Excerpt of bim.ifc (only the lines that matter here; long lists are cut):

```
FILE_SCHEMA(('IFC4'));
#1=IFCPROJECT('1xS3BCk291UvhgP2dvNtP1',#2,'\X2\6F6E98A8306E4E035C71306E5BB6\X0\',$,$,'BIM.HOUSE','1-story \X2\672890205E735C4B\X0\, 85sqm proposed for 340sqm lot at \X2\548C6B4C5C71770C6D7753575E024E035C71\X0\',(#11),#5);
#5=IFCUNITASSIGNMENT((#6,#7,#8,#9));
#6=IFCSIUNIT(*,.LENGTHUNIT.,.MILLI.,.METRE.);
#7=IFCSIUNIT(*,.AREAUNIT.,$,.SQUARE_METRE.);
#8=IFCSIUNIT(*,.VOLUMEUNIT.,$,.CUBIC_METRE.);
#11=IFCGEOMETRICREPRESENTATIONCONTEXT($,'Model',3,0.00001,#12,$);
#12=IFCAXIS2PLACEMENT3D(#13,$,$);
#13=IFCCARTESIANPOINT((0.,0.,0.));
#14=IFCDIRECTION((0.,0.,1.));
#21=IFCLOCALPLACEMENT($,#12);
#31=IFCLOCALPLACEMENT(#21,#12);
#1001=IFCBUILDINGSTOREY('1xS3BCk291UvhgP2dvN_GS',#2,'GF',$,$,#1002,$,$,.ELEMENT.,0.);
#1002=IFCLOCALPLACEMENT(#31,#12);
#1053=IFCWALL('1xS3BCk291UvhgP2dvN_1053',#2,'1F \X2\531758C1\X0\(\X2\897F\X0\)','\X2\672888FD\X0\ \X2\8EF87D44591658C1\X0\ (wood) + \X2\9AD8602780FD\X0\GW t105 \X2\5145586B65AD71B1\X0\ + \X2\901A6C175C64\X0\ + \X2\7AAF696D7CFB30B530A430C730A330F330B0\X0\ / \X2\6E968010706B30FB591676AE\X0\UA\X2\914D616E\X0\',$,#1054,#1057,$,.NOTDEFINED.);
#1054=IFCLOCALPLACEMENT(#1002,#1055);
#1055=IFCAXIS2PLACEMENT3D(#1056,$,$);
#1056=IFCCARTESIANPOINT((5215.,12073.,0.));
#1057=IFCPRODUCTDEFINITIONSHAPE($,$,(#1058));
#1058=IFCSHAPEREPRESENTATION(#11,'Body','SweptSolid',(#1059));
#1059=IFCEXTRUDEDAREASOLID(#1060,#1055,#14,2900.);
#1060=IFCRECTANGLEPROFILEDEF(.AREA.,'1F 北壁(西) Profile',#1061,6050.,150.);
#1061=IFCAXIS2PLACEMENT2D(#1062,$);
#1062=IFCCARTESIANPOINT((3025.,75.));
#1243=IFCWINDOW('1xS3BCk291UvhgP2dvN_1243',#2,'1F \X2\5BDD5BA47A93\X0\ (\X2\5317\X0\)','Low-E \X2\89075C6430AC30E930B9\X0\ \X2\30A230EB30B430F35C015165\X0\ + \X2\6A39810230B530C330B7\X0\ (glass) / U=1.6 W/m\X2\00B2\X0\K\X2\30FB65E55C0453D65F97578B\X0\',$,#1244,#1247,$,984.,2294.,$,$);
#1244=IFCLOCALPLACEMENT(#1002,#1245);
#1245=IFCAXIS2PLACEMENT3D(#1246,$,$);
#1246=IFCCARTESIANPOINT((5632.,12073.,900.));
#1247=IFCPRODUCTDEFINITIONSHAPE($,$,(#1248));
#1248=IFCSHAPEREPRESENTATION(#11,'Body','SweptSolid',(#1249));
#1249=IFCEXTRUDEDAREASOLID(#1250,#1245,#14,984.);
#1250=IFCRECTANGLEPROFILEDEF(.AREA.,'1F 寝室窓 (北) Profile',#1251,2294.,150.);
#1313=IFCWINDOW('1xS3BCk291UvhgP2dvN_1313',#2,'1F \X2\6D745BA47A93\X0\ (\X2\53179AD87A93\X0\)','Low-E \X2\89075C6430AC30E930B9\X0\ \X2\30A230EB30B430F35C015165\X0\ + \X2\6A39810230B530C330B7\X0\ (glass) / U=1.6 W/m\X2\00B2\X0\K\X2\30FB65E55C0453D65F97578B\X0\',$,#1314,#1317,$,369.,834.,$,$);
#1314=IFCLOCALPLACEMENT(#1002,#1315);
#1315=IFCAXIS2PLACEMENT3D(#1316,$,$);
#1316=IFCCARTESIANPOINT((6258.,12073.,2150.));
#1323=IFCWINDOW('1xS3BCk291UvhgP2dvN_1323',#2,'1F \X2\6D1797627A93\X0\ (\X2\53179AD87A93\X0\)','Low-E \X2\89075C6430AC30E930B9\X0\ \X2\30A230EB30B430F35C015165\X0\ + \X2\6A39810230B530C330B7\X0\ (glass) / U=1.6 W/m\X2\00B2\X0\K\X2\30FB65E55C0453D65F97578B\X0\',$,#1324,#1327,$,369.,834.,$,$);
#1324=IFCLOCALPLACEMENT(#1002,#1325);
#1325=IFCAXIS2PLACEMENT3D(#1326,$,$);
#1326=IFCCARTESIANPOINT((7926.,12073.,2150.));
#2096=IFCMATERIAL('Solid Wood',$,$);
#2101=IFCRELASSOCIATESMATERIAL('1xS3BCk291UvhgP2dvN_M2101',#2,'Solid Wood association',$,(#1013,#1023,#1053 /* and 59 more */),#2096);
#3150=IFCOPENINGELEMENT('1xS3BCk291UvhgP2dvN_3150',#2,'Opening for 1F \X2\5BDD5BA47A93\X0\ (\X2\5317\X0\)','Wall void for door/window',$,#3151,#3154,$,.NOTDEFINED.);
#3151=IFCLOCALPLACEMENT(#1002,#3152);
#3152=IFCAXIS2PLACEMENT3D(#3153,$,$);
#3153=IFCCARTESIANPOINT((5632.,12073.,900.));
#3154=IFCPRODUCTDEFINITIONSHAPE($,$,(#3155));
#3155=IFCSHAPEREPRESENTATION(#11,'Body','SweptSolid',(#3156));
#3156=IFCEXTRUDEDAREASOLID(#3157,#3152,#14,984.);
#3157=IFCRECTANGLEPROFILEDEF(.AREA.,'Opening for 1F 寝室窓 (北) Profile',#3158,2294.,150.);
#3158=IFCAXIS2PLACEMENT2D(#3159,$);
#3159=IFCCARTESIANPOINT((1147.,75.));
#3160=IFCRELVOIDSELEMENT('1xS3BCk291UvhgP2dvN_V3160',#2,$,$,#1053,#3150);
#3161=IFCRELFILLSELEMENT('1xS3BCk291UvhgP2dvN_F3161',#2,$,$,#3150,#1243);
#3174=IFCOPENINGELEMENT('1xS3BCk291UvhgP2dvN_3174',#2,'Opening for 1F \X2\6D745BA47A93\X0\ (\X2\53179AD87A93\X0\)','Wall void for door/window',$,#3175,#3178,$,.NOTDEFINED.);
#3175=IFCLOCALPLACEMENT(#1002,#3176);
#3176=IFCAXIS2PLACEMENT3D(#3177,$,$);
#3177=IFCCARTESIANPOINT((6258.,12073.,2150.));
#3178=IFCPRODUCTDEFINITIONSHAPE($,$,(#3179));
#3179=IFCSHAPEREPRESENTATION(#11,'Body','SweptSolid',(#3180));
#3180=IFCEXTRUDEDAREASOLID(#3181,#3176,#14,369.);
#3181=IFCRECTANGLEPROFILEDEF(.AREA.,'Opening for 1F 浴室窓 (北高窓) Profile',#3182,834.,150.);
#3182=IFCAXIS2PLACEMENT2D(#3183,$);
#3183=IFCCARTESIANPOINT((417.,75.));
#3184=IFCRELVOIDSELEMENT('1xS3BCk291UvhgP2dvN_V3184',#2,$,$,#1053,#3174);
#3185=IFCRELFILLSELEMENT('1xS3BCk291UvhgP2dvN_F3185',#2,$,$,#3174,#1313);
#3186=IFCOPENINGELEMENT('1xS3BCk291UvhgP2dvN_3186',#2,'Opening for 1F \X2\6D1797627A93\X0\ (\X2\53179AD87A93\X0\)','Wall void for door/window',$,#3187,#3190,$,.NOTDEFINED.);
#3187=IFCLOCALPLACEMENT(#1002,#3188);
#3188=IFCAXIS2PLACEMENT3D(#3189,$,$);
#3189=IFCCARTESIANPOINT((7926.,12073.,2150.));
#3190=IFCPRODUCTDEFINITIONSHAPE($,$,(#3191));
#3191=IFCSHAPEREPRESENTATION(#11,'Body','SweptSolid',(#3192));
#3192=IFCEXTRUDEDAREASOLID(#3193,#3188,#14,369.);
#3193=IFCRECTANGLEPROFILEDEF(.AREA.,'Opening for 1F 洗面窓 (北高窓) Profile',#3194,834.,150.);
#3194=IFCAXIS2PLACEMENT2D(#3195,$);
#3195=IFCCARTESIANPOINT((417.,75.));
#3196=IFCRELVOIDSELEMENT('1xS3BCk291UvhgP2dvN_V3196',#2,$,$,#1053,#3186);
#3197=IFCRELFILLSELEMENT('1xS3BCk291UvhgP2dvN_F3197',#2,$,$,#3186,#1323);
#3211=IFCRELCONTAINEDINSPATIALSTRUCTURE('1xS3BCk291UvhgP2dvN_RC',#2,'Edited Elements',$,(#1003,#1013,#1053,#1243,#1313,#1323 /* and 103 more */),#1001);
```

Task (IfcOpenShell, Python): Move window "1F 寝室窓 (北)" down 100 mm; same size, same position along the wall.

```python
import numpy as np
import ifcopenshell
import ifcopenshell.api.geometry
import ifcopenshell.util.placement
import ifcopenshell.util.unit

model = ifcopenshell.open("bim.ifc")
unit_scale = ifcopenshell.util.unit.calculate_unit_scale(model)

window = model.by_guid("1xS3BCk291UvhgP2dvN_1243")
opening = window.FillsVoids[0].RelatingOpeningElement
dz = -100.0

shift = np.array([0.0, 0.0, dz])
# The window is not placed relative to its opening, so move both.
for product in (opening, window):
    matrix = ifcopenshell.util.placement.get_local_placement(product.ObjectPlacement)
    matrix[:3, 3] += shift
    ifcopenshell.api.geometry.edit_object_placement(model, product=product, matrix=matrix, is_si=False)

print(f"moved by {dz * unit_scale:+.3f} m")

model.write("bim_updated.ifc")
```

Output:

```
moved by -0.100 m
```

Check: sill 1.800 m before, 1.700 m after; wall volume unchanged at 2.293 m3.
